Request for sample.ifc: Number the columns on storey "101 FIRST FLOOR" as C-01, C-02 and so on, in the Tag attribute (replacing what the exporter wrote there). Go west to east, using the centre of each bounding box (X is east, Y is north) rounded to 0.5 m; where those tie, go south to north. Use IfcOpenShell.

First a look at what the model holds.

```python
import ifcopenshell
import ifcopenshell.util.element
import ifcopenshell.util.placement

model = ifcopenshell.open("sample.ifc")
print(model.schema)
storey = next(s for s in model.by_type("IfcBuildingStorey") if s.Name == "101 FIRST FLOOR")
columns = [e for e in ifcopenshell.util.element.get_decomposition(storey) if e.is_a("IfcColumn")]
for e in sorted(columns, key=lambda e: e.id()):
    origin = ifcopenshell.util.placement.get_local_placement(e.ObjectPlacement)[:3, 3]
    print(e.id(), e.Tag, e.Name, origin.round(2) + 0.0, sep=" | ")
```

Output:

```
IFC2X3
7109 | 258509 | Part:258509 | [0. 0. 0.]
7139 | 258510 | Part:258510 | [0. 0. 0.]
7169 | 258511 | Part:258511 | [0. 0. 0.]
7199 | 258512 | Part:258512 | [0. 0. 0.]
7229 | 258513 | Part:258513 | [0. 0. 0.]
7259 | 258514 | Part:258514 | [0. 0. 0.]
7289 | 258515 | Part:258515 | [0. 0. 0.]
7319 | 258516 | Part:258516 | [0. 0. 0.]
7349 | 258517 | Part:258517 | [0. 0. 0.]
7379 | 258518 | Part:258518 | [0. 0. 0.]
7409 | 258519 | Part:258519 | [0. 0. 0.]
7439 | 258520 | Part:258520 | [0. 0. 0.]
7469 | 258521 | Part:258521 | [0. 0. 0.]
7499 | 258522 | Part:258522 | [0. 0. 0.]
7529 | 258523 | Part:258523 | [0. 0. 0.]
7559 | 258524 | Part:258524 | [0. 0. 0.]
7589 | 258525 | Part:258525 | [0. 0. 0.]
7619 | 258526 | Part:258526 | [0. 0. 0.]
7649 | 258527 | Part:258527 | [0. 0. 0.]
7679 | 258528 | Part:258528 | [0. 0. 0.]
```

```python
import ifcopenshell
import ifcopenshell.geom
import ifcopenshell.util.element
import ifcopenshell.util.shape

model = ifcopenshell.open("sample.ifc")
settings = ifcopenshell.geom.settings()
settings.set("use-world-coords", True)


def centre(element):
    shape = ifcopenshell.geom.create_shape(settings, element)
    return ifcopenshell.util.shape.get_bbox_centroid(shape.geometry)


storey = next(s for s in model.by_type("IfcBuildingStorey") if s.Name == "101 FIRST FLOOR")
columns = [e for e in ifcopenshell.util.element.get_decomposition(storey) if e.is_a("IfcColumn")]

# Insertion points can sit at a corner or the storey origin, so sort by the geometry (in metres).
centres = {e: centre(e) for e in columns}
columns.sort(key=lambda e: (round(centres[e][0] / 0.5), centres[e][1]))

for i, e in enumerate(columns, start=1):
    number = f"C-{i:02d}"
    e.Tag = number
    print(e.id(), number)

model.write("sample_rev.ifc")
```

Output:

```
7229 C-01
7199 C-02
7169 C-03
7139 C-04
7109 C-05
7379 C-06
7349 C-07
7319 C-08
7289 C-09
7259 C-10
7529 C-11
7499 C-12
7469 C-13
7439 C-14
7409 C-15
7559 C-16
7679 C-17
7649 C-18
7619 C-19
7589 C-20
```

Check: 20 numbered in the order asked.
